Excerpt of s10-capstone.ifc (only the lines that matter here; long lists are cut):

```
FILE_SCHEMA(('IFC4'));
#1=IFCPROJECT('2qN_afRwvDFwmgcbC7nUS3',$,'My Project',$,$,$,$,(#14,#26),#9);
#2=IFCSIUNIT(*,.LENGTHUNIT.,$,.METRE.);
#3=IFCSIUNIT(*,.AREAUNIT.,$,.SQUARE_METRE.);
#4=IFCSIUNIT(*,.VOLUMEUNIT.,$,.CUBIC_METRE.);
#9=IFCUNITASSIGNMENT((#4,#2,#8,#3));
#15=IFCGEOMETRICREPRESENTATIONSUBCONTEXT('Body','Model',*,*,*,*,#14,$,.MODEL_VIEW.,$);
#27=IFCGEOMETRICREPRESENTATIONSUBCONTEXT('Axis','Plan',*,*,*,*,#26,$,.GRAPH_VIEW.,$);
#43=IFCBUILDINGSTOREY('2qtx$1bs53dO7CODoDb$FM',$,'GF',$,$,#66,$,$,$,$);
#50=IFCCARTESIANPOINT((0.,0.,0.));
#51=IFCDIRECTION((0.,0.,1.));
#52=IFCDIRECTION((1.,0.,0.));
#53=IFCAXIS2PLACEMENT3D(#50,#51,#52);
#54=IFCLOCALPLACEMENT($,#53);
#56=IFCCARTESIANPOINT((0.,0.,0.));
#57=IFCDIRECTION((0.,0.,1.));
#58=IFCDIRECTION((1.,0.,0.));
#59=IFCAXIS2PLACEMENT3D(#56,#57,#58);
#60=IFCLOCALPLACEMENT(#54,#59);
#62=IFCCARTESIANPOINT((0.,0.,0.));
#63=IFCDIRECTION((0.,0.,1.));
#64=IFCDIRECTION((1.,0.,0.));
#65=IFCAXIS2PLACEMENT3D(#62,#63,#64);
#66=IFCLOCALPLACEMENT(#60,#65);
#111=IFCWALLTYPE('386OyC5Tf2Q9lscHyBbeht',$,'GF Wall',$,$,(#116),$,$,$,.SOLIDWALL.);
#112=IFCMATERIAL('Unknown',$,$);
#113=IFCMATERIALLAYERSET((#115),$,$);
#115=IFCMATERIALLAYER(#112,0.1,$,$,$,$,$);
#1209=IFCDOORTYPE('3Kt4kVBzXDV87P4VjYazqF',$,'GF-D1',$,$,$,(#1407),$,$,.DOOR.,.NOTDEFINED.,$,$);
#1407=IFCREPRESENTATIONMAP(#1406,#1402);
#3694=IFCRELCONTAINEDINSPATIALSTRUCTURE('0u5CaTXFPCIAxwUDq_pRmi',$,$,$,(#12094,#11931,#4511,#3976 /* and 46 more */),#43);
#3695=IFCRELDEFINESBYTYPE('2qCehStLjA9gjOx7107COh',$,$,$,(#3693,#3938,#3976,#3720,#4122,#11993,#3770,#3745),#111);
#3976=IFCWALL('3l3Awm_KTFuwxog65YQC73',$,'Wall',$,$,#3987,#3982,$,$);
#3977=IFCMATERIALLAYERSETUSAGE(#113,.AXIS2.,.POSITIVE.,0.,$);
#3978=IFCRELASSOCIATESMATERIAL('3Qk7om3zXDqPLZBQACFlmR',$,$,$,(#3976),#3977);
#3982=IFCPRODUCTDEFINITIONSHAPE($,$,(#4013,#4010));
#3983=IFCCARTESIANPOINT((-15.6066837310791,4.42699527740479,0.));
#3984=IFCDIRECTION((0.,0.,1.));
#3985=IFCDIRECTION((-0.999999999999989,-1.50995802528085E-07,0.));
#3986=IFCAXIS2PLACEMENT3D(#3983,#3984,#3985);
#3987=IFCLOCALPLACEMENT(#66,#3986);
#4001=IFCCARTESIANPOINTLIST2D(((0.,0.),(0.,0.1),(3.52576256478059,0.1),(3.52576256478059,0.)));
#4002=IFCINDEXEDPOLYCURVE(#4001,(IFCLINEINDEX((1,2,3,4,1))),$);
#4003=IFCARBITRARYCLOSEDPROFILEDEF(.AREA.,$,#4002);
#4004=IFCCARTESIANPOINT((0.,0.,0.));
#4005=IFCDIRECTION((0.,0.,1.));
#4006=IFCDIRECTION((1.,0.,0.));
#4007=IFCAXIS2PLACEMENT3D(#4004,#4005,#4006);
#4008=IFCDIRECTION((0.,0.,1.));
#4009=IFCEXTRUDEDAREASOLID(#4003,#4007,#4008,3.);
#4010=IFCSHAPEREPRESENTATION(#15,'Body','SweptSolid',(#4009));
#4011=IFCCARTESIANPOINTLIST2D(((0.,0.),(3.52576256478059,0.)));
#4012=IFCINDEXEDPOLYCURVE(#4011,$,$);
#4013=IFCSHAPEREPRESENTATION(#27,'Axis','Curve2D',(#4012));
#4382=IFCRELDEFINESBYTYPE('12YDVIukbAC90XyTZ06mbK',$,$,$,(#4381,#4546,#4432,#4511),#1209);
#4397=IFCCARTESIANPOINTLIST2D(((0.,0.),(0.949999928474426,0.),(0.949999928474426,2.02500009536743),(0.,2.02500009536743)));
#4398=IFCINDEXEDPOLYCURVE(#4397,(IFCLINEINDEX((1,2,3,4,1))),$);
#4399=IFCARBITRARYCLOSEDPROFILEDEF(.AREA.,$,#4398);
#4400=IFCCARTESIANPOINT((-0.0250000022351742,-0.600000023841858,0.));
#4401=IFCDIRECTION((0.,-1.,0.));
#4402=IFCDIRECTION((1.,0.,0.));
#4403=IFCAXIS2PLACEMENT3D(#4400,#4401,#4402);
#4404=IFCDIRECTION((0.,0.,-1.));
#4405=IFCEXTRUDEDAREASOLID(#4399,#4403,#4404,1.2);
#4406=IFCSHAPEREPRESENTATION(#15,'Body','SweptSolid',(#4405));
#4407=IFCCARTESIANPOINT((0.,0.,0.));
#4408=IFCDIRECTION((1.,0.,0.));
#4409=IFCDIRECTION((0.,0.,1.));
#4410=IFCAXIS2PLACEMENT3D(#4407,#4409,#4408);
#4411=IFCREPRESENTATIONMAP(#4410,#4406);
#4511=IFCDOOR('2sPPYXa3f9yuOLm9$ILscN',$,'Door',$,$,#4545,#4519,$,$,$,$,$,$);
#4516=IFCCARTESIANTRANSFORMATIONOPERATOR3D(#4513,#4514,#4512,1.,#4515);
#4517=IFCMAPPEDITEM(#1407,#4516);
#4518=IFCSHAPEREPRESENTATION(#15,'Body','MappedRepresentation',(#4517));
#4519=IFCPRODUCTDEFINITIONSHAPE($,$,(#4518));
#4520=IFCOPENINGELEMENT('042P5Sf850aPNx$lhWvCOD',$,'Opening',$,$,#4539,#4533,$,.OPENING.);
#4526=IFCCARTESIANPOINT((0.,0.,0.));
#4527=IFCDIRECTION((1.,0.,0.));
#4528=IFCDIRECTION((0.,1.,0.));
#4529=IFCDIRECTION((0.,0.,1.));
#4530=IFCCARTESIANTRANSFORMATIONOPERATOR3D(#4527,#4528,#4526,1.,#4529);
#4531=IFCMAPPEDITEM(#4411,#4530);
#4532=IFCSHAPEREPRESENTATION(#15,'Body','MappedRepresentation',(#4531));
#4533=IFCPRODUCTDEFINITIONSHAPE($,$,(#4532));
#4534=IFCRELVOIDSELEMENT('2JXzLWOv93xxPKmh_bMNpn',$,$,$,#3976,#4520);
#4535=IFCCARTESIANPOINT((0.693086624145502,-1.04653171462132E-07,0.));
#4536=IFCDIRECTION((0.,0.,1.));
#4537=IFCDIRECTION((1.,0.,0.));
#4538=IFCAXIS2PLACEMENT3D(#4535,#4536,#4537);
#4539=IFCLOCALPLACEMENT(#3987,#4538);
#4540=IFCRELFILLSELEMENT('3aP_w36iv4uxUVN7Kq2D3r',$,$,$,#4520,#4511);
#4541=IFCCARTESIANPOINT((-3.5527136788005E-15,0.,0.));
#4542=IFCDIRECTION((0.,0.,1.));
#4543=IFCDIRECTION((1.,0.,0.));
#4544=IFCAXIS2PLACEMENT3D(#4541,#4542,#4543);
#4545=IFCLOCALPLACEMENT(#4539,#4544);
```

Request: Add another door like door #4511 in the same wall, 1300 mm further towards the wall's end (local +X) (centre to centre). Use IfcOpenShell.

```python
import ifcopenshell
import ifcopenshell.api.feature
import ifcopenshell.api.geometry
import ifcopenshell.api.root
import ifcopenshell.geom
import ifcopenshell.util.element
import ifcopenshell.util.placement
import ifcopenshell.util.shape

model = ifcopenshell.open("s10-capstone.ifc")
settings = ifcopenshell.geom.settings()


def volume(element):
    """Net volume in cubic metres, openings subtracted."""
    shape = ifcopenshell.geom.create_shape(settings, element)
    return ifcopenshell.util.shape.get_volume(shape.geometry)


door = model.by_guid("2sPPYXa3f9yuOLm9$ILscN")
opening = door.FillsVoids[0].RelatingOpeningElement
wall = opening.VoidsElements[0].RelatingBuildingElement
before = volume(wall)
shift = ifcopenshell.util.placement.get_local_placement(wall.ObjectPlacement)[:3, 0] * 1.3

# copy_class copies the void relationship, type, container and properties, but no geometry.
new_opening = ifcopenshell.api.root.copy_class(model, product=opening)
new_opening.Representation = ifcopenshell.util.element.copy_deep(
    model, opening.Representation, exclude=["IfcGeometricRepresentationContext", "IfcRepresentationMap"]
)
new_door = ifcopenshell.api.root.copy_class(model, product=door)
new_door.Representation = ifcopenshell.util.element.copy_deep(
    model, door.Representation, exclude=["IfcGeometricRepresentationContext", "IfcRepresentationMap"]
)
ifcopenshell.api.feature.add_filling(model, opening=new_opening, element=new_door)

for old, new in ((opening, new_opening), (door, new_door)):
    matrix = ifcopenshell.util.placement.get_local_placement(old.ObjectPlacement)
    matrix[:3, 3] += shift
    ifcopenshell.api.geometry.edit_object_placement(model, product=new, matrix=matrix, is_si=False)

after = volume(wall)

print(f"wall volume {before:.3f} -> {after:.3f} m3")

model.write("s10-capstone_rev.ifc")
```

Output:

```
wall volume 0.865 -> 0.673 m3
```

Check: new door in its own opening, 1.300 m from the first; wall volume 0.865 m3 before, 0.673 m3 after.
